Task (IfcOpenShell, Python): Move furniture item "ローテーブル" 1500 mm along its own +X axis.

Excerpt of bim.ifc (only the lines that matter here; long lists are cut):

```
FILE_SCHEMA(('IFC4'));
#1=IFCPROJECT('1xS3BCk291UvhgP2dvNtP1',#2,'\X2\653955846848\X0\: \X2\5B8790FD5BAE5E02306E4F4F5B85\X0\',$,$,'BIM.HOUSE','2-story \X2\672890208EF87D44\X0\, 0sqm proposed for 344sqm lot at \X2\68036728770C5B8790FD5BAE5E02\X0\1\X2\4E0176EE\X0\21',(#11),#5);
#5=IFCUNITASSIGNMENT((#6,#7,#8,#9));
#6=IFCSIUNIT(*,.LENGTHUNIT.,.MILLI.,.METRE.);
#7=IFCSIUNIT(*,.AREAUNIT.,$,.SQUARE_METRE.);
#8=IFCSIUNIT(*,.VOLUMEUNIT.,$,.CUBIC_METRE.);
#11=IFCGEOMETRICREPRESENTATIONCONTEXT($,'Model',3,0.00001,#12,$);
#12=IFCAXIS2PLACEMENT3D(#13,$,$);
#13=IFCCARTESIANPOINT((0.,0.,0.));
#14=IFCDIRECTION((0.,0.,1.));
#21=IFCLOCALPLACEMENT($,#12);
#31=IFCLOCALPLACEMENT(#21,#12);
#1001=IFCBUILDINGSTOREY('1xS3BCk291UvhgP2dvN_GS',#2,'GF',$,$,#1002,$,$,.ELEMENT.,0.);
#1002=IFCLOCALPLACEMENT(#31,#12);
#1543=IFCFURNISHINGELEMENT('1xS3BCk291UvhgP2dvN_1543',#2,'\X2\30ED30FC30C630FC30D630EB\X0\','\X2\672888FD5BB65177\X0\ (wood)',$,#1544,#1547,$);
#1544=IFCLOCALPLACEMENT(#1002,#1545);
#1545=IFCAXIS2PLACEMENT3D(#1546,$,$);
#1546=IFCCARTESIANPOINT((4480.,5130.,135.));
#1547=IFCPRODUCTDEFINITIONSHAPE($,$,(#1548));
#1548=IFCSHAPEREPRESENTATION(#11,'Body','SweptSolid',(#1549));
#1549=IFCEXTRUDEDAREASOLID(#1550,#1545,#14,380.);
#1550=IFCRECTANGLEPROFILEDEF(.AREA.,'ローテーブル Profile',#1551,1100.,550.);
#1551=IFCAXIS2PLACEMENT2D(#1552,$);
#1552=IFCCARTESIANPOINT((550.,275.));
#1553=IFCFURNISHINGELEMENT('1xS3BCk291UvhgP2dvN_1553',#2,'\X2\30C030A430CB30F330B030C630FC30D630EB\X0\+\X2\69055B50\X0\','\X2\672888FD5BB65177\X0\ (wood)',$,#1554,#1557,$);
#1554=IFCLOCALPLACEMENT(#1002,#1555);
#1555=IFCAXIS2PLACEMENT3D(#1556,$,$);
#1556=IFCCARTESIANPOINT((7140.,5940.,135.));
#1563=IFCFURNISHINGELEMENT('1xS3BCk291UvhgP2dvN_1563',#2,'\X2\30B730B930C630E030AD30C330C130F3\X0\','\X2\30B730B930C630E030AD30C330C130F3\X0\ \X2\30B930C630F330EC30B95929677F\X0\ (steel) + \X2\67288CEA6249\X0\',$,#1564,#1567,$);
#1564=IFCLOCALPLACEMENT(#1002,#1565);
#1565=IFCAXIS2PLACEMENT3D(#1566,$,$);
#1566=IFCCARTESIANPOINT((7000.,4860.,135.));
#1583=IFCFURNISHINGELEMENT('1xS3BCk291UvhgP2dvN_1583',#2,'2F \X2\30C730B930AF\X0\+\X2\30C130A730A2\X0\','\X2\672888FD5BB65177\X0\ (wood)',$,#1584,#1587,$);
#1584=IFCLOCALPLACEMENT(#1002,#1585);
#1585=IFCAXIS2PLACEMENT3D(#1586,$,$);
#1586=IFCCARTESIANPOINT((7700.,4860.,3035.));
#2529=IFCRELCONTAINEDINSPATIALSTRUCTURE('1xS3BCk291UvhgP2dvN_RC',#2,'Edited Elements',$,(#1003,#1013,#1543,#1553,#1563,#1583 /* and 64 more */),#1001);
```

```python
import ifcopenshell
import ifcopenshell.api.geometry
import ifcopenshell.util.placement

model = ifcopenshell.open("bim.ifc")

item = model.by_id(1543)
matrix = ifcopenshell.util.placement.get_local_placement(item.ObjectPlacement)
matrix[:3, 3] += matrix[:3, 0] * 1500.0
ifcopenshell.api.geometry.edit_object_placement(model, product=item, matrix=matrix, is_si=False)

print(ifcopenshell.util.placement.get_local_placement(item.ObjectPlacement).round(3) + 0.0)

model.write("bim_updated.ifc")
```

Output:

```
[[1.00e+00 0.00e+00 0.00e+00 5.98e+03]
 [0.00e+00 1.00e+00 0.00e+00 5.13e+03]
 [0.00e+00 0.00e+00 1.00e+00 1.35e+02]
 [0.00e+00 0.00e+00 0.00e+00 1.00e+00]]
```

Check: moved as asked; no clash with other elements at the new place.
